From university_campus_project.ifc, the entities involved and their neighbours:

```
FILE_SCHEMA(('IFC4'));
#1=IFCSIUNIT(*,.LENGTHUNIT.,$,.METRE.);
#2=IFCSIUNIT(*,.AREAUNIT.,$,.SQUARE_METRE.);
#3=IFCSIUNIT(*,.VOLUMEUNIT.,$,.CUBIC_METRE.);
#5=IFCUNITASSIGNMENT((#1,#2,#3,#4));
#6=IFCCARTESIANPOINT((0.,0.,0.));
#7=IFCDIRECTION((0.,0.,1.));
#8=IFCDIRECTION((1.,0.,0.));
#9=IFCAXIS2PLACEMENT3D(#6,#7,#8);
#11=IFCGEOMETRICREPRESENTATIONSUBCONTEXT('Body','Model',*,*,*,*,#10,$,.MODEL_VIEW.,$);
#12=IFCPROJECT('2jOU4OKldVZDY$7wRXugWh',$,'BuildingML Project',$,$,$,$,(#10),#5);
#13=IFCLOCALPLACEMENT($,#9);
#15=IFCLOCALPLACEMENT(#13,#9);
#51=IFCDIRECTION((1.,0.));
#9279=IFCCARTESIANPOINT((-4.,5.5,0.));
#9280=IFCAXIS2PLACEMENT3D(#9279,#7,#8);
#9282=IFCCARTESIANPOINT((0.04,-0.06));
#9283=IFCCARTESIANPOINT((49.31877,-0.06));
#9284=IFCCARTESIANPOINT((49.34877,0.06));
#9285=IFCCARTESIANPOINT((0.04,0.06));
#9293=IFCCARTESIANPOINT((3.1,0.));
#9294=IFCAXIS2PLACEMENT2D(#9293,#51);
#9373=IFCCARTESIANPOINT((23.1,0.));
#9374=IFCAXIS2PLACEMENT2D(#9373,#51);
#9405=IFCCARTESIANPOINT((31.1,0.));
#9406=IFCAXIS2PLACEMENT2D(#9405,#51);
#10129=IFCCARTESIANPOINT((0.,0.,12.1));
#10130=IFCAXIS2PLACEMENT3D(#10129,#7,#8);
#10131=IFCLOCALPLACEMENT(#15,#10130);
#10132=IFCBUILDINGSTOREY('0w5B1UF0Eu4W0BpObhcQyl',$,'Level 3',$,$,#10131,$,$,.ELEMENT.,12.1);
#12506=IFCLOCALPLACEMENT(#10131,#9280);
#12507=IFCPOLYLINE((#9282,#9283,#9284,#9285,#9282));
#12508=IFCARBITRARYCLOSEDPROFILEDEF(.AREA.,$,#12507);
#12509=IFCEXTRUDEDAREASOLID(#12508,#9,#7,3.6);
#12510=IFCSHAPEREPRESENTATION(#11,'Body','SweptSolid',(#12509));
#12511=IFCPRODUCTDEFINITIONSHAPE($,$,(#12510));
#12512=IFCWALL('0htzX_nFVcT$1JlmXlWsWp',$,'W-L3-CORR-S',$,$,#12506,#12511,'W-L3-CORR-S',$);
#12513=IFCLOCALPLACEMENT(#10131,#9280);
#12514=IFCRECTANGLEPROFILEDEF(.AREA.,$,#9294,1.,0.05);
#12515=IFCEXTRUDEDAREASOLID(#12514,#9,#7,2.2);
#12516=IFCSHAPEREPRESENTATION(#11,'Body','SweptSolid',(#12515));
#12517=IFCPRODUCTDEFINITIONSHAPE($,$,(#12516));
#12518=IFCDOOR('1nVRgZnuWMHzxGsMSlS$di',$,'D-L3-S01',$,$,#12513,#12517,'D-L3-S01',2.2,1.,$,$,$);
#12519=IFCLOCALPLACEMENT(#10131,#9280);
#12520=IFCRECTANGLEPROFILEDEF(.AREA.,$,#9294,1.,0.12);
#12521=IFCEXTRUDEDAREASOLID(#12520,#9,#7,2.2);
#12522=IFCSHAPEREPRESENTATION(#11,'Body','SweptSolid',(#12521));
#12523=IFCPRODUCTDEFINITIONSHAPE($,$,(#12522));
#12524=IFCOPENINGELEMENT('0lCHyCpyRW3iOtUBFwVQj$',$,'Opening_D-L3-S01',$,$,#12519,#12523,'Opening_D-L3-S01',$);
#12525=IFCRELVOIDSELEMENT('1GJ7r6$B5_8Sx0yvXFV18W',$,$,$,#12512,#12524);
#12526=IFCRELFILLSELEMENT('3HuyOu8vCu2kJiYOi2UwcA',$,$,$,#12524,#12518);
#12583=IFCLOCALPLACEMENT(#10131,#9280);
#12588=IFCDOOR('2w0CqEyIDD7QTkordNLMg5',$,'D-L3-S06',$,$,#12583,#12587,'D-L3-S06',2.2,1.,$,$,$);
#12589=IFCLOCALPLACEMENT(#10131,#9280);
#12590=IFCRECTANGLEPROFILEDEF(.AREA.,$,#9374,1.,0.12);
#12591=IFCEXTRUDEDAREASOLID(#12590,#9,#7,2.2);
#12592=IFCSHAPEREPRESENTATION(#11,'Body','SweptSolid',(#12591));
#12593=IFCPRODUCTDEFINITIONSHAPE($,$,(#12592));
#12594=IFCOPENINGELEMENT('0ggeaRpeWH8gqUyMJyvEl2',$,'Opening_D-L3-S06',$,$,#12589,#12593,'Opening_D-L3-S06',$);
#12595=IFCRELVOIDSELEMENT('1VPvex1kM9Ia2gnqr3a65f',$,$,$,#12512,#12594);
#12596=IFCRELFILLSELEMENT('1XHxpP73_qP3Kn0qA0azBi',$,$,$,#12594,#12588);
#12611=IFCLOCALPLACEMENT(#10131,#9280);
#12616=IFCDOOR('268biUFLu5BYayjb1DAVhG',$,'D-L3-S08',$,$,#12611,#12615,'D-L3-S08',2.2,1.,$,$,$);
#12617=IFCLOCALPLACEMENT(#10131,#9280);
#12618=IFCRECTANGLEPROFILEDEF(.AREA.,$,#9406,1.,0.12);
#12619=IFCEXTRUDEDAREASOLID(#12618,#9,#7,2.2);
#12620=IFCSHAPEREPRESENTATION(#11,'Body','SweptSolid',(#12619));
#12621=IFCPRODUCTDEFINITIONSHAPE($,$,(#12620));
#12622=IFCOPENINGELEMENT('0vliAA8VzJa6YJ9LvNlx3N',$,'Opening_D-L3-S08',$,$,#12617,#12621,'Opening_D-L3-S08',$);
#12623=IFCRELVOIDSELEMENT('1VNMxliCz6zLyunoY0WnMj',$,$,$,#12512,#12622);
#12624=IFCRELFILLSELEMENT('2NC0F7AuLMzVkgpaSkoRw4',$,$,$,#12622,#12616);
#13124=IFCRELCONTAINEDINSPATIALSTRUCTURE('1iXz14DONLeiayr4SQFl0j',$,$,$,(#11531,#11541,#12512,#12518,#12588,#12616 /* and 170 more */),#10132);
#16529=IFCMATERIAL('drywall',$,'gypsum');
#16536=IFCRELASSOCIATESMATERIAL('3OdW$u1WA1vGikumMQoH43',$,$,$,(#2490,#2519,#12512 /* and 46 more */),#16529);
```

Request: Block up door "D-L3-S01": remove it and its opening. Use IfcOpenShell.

```python
import ifcopenshell
import ifcopenshell.api.feature
import ifcopenshell.api.root
import ifcopenshell.geom
import ifcopenshell.util.shape

model = ifcopenshell.open("university_campus_project.ifc")
settings = ifcopenshell.geom.settings()


def volume(element):
    """Net volume in cubic metres, openings subtracted."""
    shape = ifcopenshell.geom.create_shape(settings, element)
    return ifcopenshell.util.shape.get_volume(shape.geometry)


door = model.by_guid("1nVRgZnuWMHzxGsMSlS$di")
opening = door.FillsVoids[0].RelatingOpeningElement
wall = opening.VoidsElements[0].RelatingBuildingElement
before = volume(wall)

ifcopenshell.api.root.remove_product(model, product=door)
ifcopenshell.api.feature.remove_feature(model, feature=opening)

after = volume(wall)

print(f"wall volume {before:.3f} -> {after:.3f} m3")

model.write("university_campus_project_v2.ifc")
```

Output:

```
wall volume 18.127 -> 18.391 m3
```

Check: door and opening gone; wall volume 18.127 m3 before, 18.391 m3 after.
